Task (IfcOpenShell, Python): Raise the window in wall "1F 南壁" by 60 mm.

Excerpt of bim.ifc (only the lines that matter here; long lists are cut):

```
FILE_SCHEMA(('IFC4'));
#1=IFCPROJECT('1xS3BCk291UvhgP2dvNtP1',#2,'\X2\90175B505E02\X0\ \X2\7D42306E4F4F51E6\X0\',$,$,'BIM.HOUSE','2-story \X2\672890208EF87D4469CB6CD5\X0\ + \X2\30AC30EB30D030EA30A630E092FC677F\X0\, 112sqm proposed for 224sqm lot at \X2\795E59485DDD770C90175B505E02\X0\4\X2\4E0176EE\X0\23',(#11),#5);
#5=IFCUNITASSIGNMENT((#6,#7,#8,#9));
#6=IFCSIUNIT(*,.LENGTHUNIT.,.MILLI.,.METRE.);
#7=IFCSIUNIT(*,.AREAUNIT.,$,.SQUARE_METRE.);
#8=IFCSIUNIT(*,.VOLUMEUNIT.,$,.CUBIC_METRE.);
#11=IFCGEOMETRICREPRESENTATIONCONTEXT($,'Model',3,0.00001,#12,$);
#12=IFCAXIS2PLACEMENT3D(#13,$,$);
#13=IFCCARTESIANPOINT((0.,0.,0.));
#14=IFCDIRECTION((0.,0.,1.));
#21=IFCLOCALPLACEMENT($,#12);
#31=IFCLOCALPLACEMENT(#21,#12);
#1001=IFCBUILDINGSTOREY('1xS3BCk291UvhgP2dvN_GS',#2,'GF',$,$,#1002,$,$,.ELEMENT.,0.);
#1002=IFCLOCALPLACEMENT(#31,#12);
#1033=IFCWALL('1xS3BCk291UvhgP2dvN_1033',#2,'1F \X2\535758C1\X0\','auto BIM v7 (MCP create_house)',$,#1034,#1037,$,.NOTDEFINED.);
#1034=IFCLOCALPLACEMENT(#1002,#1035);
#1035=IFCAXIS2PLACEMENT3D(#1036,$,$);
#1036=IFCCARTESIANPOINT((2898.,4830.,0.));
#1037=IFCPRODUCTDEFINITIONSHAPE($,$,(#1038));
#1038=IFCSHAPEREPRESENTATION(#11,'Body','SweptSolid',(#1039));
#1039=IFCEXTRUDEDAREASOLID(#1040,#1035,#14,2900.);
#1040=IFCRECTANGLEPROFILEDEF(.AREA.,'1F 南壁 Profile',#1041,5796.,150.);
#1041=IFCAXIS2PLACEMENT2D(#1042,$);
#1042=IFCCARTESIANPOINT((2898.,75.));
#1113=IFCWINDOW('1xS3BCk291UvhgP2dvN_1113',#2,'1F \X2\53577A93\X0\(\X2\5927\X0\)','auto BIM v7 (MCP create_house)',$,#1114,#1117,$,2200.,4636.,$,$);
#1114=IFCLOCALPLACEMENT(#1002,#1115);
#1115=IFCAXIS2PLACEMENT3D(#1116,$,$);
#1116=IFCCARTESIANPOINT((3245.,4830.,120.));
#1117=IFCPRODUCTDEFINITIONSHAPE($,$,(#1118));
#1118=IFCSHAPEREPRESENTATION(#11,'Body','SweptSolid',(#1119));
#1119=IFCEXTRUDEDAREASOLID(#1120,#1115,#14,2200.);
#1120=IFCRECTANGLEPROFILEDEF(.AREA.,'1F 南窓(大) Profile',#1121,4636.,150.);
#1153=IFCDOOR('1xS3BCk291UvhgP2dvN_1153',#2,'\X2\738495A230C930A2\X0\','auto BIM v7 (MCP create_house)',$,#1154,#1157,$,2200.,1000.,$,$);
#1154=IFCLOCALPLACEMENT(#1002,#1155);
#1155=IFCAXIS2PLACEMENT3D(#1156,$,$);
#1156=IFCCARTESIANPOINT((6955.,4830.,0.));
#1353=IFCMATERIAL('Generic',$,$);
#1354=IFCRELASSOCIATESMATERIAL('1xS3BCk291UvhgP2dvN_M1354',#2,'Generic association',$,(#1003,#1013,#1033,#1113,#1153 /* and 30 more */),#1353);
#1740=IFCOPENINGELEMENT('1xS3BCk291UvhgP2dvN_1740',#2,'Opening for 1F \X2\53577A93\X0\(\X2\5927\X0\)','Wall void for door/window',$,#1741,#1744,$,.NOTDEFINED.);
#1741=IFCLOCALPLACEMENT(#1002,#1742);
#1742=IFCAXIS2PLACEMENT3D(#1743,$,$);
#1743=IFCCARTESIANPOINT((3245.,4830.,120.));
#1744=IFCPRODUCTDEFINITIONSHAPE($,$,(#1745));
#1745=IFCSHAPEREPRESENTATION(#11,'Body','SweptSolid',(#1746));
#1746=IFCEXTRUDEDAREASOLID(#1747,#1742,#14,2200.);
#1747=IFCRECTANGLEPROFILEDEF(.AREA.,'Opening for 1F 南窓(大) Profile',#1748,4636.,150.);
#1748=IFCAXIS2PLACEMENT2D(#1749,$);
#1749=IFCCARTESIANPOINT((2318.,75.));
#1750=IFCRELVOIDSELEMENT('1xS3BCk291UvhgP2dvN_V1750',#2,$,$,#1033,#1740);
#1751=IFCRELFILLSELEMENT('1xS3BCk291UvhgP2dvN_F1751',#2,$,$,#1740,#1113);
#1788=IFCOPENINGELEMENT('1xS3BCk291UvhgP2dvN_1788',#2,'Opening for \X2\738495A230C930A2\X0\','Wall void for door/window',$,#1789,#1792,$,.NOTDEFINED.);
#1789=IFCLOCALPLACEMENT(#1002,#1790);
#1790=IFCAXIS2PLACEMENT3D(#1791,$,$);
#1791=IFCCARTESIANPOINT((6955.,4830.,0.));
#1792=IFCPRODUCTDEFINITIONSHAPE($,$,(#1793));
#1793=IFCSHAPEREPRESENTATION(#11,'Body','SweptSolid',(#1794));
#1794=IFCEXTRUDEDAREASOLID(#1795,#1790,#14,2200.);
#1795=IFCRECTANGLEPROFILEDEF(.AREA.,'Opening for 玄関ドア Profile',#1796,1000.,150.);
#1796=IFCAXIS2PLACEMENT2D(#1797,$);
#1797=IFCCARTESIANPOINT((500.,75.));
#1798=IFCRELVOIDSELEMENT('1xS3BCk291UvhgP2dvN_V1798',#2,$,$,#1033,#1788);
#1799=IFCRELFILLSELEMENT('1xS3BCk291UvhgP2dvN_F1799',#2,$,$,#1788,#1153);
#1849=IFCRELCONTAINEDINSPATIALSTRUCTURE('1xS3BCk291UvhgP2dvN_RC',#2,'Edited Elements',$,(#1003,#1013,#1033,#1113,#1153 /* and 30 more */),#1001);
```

```python
import numpy as np
import ifcopenshell
import ifcopenshell.api.geometry
import ifcopenshell.util.placement
import ifcopenshell.util.unit

model = ifcopenshell.open("bim.ifc")
unit_scale = ifcopenshell.util.unit.calculate_unit_scale(model)

window = model.by_guid("1xS3BCk291UvhgP2dvN_1113")
opening = window.FillsVoids[0].RelatingOpeningElement
dz = 0.06 / unit_scale

shift = np.array([0.0, 0.0, dz])
# The window is not placed relative to its opening, so move both.
for product in (opening, window):
    matrix = ifcopenshell.util.placement.get_local_placement(product.ObjectPlacement)
    matrix[:3, 3] += shift
    ifcopenshell.api.geometry.edit_object_placement(model, product=product, matrix=matrix, is_si=False)

print(f"moved by {dz * unit_scale:+.3f} m")

model.write("bim_edited.ifc")
```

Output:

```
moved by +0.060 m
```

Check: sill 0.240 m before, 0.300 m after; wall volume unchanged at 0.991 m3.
